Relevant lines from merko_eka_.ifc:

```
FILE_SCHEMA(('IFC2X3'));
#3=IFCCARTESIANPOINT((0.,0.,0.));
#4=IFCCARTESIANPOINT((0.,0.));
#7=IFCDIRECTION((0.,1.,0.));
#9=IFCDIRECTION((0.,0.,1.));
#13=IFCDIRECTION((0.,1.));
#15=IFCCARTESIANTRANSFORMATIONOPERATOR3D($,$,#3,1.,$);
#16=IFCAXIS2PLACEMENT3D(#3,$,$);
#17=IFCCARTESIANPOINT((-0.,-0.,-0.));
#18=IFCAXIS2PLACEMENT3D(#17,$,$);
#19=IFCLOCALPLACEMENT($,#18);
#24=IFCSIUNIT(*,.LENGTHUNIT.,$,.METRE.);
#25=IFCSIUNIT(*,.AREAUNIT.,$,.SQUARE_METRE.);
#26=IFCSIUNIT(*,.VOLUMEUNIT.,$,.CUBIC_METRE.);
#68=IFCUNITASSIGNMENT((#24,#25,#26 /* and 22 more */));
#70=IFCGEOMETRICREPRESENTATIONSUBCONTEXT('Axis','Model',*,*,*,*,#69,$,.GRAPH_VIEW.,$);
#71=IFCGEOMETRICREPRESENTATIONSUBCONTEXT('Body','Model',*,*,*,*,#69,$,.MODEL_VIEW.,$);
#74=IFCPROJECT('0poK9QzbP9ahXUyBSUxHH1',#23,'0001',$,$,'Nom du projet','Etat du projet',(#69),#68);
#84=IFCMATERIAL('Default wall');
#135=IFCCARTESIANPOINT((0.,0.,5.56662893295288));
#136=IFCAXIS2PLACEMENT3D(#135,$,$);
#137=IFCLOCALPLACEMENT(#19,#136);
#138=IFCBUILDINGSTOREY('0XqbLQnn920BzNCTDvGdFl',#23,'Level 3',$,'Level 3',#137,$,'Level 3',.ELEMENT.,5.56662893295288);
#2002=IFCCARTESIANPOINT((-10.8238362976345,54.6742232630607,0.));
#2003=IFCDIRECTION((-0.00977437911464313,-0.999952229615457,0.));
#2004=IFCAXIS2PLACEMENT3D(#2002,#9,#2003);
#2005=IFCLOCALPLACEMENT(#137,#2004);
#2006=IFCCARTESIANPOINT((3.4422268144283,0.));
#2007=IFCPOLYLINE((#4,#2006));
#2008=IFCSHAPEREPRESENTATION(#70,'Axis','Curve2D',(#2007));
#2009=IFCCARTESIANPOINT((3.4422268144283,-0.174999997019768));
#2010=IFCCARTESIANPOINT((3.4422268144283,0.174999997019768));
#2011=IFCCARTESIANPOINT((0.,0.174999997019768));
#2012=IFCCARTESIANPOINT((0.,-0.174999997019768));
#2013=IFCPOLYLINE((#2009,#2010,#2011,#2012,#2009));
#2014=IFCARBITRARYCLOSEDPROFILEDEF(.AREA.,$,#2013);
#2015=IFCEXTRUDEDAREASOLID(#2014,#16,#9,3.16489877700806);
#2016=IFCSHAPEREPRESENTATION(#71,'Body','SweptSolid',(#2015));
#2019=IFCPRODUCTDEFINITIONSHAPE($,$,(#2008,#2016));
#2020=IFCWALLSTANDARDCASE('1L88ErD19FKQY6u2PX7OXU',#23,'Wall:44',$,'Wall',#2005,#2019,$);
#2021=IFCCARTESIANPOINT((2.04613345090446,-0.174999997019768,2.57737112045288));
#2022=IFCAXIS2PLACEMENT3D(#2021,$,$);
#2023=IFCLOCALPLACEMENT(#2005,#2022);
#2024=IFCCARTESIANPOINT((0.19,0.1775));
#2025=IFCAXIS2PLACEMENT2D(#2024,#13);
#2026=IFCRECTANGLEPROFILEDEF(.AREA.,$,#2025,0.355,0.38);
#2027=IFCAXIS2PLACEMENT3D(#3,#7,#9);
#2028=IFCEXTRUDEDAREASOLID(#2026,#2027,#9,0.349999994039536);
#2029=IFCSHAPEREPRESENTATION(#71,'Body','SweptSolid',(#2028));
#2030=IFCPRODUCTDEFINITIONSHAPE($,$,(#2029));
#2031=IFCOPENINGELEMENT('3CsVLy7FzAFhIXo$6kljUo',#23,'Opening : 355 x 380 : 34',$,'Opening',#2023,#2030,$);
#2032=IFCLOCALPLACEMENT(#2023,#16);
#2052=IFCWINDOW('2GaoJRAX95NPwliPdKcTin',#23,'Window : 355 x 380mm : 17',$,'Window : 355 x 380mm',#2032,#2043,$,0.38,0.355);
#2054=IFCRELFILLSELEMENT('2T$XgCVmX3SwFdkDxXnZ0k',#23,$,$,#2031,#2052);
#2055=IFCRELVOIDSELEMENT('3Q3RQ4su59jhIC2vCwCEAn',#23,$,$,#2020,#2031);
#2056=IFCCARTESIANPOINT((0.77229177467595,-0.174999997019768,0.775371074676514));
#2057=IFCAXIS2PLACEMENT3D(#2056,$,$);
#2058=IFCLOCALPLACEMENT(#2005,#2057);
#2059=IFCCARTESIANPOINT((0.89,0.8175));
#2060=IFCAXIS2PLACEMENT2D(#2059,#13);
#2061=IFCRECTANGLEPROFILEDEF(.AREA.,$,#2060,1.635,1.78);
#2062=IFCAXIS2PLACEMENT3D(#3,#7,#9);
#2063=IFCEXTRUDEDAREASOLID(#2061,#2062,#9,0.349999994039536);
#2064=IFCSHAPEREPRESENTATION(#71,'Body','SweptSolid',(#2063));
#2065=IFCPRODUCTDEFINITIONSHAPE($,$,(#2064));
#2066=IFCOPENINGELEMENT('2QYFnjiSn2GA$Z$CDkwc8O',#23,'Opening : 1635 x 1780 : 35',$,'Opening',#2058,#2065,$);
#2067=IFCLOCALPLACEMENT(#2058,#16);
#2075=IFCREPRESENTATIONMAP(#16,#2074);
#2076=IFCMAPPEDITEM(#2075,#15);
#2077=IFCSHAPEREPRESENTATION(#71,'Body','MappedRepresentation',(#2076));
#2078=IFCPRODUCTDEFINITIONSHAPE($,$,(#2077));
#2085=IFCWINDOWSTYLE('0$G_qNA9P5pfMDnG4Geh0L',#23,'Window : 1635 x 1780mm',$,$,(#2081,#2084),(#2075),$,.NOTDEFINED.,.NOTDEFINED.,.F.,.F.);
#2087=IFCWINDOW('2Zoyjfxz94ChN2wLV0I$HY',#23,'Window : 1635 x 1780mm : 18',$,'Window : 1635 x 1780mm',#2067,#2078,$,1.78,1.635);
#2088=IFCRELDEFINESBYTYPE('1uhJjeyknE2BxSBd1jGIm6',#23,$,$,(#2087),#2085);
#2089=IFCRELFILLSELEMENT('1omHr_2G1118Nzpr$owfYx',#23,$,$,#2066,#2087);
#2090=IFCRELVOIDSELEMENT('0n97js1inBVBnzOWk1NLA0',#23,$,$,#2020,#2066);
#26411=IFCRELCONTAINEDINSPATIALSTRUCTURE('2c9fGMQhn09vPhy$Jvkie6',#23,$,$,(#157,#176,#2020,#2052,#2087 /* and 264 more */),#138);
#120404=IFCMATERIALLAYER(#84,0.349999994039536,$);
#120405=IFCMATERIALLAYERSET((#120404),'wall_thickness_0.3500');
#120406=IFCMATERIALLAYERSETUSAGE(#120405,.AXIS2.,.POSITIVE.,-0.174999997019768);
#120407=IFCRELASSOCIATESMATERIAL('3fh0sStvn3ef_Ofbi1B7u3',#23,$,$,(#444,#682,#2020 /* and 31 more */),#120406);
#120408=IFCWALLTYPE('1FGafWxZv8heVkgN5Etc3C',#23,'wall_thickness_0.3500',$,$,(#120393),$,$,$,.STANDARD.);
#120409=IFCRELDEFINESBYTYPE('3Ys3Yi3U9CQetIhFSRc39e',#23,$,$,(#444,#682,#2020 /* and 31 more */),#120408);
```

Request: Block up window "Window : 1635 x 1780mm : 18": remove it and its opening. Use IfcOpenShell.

```python
import ifcopenshell
import ifcopenshell.api.feature
import ifcopenshell.api.root
import ifcopenshell.geom
import ifcopenshell.util.shape

model = ifcopenshell.open("merko_eka_.ifc")
settings = ifcopenshell.geom.settings()


def volume(element):
    """Net volume in cubic metres, openings subtracted."""
    shape = ifcopenshell.geom.create_shape(settings, element)
    return ifcopenshell.util.shape.get_volume(shape.geometry)


window = model.by_guid("2Zoyjfxz94ChN2wLV0I$HY")
opening = window.FillsVoids[0].RelatingOpeningElement
wall = opening.VoidsElements[0].RelatingBuildingElement
before = volume(wall)

ifcopenshell.api.root.remove_product(model, product=window)
ifcopenshell.api.feature.remove_feature(model, feature=opening)

after = volume(wall)

print(f"wall volume {before:.3f} -> {after:.3f} m3")

model.write("merko_eka_-out.ifc")
```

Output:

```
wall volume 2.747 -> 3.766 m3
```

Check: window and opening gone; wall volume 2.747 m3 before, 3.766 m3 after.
